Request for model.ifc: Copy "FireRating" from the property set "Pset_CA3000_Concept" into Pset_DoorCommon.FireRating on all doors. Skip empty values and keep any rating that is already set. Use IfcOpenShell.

First a look at what the model holds.

```python
import ifcopenshell
import ifcopenshell.util.element

model = ifcopenshell.open("model.ifc")
print(model.schema)
doors = model.by_type("IfcDoor")
print(len(doors), "doors")
for e in doors[:8]:
    source = ifcopenshell.util.element.get_pset(e, "Pset_CA3000_Concept", "FireRating")
    target = ifcopenshell.util.element.get_pset(e, "Pset_DoorCommon", "FireRating")
    print(e.id(), repr(source), repr(target), sep=" | ")
```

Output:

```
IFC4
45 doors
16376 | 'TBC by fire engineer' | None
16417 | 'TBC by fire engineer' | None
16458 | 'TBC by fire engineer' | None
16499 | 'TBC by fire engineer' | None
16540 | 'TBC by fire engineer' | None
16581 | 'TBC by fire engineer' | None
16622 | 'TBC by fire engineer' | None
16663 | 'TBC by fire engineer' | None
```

```python
import ifcopenshell
import ifcopenshell.api.pset
import ifcopenshell.util.element

model = ifcopenshell.open("model.ifc")

count = 0
for e in model.by_type("IfcDoor"):
    value = ifcopenshell.util.element.get_pset(e, "Pset_CA3000_Concept", "FireRating")
    current = ifcopenshell.util.element.get_pset(e, "Pset_DoorCommon", "FireRating")
    if not value or not value.strip() or current:
        continue
    # add_pset returns the element's existing set when there is one.
    pset = ifcopenshell.api.pset.add_pset(model, product=e, name="Pset_DoorCommon")
    ifcopenshell.api.pset.edit_pset(model, pset=pset, properties={"FireRating": value})
    count += 1

print(count, "doors updated")

model.write("model_edited.ifc")
```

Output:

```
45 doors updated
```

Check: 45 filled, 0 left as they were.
